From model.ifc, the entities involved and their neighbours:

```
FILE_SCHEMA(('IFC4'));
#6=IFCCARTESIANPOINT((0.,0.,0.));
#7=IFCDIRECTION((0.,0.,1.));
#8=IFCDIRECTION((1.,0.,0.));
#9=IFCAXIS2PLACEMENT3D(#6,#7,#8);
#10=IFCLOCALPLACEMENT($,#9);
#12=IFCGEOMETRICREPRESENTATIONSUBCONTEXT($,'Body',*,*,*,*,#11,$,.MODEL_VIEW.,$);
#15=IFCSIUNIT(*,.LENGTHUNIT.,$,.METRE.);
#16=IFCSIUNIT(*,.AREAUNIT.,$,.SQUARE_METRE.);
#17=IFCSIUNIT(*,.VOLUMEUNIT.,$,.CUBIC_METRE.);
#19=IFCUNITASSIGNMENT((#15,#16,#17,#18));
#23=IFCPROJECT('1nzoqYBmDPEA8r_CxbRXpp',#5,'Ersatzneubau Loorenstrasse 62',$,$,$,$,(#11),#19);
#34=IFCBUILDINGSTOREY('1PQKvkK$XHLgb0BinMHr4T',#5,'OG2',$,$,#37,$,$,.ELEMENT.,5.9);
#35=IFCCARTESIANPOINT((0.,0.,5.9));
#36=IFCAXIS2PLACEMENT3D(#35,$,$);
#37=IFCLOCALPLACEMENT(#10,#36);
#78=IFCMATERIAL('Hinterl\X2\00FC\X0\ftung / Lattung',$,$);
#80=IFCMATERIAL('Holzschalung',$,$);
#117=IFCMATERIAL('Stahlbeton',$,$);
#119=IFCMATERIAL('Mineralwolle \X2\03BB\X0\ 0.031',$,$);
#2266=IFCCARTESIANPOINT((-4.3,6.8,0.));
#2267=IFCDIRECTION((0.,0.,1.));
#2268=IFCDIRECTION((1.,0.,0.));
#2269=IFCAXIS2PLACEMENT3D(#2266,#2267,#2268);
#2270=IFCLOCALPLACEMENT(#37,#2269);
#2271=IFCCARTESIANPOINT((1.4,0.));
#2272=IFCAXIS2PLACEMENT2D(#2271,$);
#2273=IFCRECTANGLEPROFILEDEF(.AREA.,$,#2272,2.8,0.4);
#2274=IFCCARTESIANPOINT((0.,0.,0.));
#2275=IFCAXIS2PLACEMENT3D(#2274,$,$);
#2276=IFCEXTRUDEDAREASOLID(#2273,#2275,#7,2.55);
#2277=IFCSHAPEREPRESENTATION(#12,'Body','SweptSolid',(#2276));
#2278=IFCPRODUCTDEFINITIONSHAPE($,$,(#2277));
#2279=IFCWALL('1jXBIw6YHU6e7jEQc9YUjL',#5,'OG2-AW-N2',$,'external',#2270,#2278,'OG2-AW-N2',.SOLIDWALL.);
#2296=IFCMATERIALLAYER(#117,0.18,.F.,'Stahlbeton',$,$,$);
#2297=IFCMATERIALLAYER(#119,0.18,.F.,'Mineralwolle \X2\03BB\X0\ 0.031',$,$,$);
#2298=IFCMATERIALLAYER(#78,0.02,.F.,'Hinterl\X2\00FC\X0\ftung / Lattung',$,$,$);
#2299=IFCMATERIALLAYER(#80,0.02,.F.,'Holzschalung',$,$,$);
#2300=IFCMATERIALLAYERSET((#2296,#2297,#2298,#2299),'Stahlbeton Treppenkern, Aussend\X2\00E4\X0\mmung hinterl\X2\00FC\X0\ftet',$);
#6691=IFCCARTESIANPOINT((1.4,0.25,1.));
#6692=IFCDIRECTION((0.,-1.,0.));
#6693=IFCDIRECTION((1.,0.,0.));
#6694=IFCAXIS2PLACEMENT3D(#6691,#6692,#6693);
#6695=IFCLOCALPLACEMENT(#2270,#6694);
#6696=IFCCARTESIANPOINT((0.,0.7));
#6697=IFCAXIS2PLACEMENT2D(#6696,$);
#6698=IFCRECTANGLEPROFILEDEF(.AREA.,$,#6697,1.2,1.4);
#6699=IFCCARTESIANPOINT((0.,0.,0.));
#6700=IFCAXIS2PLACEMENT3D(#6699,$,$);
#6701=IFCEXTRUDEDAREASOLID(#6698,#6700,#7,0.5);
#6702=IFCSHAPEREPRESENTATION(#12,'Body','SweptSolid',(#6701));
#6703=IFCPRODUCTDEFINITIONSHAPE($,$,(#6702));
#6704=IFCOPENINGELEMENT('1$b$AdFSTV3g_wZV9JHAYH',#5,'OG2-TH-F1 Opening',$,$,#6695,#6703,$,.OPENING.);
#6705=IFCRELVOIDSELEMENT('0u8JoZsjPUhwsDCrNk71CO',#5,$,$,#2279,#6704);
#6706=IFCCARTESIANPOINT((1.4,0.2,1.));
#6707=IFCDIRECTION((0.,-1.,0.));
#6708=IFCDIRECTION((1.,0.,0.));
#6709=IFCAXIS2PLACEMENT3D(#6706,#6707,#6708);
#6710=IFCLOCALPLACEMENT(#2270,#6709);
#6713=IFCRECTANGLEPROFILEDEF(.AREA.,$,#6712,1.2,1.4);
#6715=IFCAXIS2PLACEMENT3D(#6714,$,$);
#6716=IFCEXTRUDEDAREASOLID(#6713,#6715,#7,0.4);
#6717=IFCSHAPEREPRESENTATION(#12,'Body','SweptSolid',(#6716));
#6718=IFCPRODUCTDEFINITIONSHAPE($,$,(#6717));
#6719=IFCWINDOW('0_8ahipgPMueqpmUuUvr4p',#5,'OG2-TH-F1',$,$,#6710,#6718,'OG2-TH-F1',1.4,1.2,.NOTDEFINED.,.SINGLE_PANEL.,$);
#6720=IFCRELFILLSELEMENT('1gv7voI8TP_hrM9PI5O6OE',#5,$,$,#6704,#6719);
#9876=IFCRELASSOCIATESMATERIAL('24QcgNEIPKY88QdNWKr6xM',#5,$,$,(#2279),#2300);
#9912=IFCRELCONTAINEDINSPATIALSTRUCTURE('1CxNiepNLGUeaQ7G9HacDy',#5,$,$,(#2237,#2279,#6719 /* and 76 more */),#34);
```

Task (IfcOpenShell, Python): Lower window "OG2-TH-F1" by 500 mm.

```python
import numpy as np
import ifcopenshell
import ifcopenshell.api.geometry
import ifcopenshell.util.placement
import ifcopenshell.util.unit

model = ifcopenshell.open("model.ifc")
unit_scale = ifcopenshell.util.unit.calculate_unit_scale(model)

window = model.by_guid("0_8ahipgPMueqpmUuUvr4p")
opening = window.FillsVoids[0].RelatingOpeningElement
dz = -0.5

shift = np.array([0.0, 0.0, dz])
# The window is not placed relative to its opening, so move both.
for product in (opening, window):
    matrix = ifcopenshell.util.placement.get_local_placement(product.ObjectPlacement)
    matrix[:3, 3] += shift
    ifcopenshell.api.geometry.edit_object_placement(model, product=product, matrix=matrix, is_si=False)

print(f"moved by {dz * unit_scale:+.3f} m")

model.write("model-out.ifc")
```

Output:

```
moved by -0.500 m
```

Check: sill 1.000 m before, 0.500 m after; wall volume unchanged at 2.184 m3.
